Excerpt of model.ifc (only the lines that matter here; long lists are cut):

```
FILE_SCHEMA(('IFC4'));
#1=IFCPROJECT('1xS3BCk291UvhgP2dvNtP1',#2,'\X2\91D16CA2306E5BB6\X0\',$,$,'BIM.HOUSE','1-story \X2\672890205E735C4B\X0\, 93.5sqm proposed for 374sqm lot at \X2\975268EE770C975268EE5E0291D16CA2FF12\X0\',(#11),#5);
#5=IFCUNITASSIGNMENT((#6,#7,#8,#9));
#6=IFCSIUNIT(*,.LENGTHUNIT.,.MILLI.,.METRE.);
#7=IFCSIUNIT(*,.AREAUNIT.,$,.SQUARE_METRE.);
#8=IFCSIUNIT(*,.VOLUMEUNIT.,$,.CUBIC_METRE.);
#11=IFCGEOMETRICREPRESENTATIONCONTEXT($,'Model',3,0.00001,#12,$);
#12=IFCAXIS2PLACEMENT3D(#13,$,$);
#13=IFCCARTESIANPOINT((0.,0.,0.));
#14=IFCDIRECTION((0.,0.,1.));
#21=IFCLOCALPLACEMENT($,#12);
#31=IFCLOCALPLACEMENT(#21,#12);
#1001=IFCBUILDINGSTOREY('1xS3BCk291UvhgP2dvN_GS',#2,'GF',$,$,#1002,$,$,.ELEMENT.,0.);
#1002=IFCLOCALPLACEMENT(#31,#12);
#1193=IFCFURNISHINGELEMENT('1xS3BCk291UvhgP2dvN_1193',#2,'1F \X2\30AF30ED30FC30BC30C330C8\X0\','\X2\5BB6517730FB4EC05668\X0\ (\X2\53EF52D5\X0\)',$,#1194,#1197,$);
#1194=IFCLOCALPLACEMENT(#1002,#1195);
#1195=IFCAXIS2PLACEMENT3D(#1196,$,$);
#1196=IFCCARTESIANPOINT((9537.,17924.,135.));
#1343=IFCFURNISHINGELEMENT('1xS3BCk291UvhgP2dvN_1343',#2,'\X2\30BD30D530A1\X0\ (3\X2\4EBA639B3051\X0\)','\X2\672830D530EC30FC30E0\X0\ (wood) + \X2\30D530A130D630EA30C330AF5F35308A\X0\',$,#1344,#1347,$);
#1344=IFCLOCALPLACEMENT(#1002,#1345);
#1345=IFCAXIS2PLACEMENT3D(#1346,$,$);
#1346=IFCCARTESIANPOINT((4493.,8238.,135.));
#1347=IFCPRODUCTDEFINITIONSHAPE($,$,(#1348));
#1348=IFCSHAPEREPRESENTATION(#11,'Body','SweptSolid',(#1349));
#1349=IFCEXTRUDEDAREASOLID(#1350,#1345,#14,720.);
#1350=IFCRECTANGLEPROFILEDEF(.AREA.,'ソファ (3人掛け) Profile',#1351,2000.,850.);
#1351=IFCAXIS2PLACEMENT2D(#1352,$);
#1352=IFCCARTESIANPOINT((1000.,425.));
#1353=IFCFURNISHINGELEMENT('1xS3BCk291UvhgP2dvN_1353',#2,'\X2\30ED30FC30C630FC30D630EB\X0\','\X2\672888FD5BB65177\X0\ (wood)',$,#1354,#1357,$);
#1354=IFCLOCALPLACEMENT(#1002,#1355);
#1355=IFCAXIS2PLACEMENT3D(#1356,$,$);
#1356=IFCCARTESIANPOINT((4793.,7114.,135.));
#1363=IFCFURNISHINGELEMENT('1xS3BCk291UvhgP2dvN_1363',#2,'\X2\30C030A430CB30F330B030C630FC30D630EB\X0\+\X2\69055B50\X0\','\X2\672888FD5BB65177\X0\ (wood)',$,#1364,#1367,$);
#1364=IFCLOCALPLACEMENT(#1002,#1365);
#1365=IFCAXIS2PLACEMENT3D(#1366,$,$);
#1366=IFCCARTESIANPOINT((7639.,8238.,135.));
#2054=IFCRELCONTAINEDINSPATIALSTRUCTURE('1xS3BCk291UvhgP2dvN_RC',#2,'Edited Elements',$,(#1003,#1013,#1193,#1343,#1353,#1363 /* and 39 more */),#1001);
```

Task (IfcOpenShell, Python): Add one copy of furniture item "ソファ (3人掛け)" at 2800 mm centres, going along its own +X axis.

```python
import ifcopenshell
import ifcopenshell.api.geometry
import ifcopenshell.api.root
import ifcopenshell.util.element
import ifcopenshell.util.placement
import ifcopenshell.util.unit

model = ifcopenshell.open("model.ifc")
unit_scale = ifcopenshell.util.unit.calculate_unit_scale(model)


def reuse_history(source, copy):
    """copy_class also copies each property set's owner history, people and application; keep the originals."""
    for rel in copy.IsDefinedBy:
        if rel.is_a("IfcRelDefinesByProperties") and (history := rel.RelatingPropertyDefinition.OwnerHistory):
            rel.RelatingPropertyDefinition.OwnerHistory = source.OwnerHistory
            ifcopenshell.util.element.remove_deep2(model, history)


source = model.by_guid("1xS3BCk291UvhgP2dvN_1343")
base = ifcopenshell.util.placement.get_local_placement(source.ObjectPlacement)
step = base[:3, 0] * 2.8 / unit_scale

for i in range(1, 2):
    copy = ifcopenshell.api.root.copy_class(model, product=source)
    copy.Representation = ifcopenshell.util.element.copy_deep(
        model, source.Representation, exclude=["IfcGeometricRepresentationContext", "IfcRepresentationMap"]
    )
    reuse_history(source, copy)
    matrix = base.copy()
    matrix[:3, 3] += i * step
    print("added at", matrix[:3, 3].round(3) + 0.0)
    ifcopenshell.api.geometry.edit_object_placement(model, product=copy, matrix=matrix, is_si=False)

model.write("model_edited.ifc")
```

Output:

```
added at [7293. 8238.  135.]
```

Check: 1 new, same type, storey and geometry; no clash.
